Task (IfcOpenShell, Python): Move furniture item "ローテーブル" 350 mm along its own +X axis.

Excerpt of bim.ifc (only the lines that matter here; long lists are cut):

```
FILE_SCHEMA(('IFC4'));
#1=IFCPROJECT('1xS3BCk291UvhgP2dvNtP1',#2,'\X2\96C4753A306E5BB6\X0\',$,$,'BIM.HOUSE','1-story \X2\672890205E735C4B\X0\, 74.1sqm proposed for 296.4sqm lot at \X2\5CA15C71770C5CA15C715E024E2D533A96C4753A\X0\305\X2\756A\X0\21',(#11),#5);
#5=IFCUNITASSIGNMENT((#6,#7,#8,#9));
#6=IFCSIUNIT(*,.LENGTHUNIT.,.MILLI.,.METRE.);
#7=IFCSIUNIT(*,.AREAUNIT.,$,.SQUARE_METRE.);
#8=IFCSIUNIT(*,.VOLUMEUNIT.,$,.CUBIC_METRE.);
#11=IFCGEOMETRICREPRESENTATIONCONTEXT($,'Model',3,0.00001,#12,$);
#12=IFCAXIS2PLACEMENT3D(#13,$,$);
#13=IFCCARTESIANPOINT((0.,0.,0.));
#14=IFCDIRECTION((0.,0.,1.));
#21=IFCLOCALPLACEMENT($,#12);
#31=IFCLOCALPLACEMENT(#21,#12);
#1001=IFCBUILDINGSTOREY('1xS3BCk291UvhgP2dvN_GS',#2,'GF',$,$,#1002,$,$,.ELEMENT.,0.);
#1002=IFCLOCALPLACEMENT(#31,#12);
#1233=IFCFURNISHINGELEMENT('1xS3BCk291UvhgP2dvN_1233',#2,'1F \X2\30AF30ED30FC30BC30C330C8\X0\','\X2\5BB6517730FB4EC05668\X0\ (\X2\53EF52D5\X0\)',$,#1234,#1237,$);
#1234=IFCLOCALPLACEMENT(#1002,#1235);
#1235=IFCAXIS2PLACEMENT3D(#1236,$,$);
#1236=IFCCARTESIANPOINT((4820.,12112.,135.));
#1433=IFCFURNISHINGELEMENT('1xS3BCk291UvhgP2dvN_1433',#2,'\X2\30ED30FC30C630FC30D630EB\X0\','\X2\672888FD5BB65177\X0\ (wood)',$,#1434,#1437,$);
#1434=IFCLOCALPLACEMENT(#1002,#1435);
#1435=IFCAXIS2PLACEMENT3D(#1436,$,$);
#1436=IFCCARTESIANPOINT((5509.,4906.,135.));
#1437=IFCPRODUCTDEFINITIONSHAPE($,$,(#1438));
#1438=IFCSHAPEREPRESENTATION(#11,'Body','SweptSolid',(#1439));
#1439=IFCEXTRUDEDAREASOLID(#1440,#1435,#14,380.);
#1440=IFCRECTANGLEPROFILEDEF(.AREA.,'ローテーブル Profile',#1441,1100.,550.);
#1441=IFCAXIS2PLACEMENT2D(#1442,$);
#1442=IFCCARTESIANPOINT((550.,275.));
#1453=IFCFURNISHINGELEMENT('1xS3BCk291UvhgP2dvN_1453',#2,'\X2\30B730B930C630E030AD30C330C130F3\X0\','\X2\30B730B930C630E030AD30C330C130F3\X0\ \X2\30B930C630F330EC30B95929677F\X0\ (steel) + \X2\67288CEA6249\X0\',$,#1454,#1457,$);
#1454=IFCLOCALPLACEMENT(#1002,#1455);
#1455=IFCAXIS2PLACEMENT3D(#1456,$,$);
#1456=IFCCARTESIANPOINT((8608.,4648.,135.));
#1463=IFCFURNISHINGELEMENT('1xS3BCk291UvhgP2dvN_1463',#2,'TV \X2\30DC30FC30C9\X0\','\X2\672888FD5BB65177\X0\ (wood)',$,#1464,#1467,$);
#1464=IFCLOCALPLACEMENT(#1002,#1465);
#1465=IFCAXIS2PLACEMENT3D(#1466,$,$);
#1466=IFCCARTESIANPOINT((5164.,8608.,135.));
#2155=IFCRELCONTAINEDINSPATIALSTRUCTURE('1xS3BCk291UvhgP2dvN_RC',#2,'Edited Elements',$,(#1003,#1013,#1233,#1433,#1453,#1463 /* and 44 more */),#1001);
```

```python
import ifcopenshell
import ifcopenshell.api.geometry
import ifcopenshell.util.placement
import ifcopenshell.util.unit

model = ifcopenshell.open("bim.ifc")
unit_scale = ifcopenshell.util.unit.calculate_unit_scale(model)

item = model.by_guid("1xS3BCk291UvhgP2dvN_1433")
matrix = ifcopenshell.util.placement.get_local_placement(item.ObjectPlacement)
matrix[:3, 3] += matrix[:3, 0] * 0.35 / unit_scale
ifcopenshell.api.geometry.edit_object_placement(model, product=item, matrix=matrix, is_si=False)

print(ifcopenshell.util.placement.get_local_placement(item.ObjectPlacement).round(3) + 0.0)

model.write("bim-out.ifc")
```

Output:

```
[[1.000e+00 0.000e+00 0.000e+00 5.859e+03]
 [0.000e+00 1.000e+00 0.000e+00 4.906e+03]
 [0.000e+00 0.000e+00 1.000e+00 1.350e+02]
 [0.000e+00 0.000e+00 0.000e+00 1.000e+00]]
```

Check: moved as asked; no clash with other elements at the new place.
